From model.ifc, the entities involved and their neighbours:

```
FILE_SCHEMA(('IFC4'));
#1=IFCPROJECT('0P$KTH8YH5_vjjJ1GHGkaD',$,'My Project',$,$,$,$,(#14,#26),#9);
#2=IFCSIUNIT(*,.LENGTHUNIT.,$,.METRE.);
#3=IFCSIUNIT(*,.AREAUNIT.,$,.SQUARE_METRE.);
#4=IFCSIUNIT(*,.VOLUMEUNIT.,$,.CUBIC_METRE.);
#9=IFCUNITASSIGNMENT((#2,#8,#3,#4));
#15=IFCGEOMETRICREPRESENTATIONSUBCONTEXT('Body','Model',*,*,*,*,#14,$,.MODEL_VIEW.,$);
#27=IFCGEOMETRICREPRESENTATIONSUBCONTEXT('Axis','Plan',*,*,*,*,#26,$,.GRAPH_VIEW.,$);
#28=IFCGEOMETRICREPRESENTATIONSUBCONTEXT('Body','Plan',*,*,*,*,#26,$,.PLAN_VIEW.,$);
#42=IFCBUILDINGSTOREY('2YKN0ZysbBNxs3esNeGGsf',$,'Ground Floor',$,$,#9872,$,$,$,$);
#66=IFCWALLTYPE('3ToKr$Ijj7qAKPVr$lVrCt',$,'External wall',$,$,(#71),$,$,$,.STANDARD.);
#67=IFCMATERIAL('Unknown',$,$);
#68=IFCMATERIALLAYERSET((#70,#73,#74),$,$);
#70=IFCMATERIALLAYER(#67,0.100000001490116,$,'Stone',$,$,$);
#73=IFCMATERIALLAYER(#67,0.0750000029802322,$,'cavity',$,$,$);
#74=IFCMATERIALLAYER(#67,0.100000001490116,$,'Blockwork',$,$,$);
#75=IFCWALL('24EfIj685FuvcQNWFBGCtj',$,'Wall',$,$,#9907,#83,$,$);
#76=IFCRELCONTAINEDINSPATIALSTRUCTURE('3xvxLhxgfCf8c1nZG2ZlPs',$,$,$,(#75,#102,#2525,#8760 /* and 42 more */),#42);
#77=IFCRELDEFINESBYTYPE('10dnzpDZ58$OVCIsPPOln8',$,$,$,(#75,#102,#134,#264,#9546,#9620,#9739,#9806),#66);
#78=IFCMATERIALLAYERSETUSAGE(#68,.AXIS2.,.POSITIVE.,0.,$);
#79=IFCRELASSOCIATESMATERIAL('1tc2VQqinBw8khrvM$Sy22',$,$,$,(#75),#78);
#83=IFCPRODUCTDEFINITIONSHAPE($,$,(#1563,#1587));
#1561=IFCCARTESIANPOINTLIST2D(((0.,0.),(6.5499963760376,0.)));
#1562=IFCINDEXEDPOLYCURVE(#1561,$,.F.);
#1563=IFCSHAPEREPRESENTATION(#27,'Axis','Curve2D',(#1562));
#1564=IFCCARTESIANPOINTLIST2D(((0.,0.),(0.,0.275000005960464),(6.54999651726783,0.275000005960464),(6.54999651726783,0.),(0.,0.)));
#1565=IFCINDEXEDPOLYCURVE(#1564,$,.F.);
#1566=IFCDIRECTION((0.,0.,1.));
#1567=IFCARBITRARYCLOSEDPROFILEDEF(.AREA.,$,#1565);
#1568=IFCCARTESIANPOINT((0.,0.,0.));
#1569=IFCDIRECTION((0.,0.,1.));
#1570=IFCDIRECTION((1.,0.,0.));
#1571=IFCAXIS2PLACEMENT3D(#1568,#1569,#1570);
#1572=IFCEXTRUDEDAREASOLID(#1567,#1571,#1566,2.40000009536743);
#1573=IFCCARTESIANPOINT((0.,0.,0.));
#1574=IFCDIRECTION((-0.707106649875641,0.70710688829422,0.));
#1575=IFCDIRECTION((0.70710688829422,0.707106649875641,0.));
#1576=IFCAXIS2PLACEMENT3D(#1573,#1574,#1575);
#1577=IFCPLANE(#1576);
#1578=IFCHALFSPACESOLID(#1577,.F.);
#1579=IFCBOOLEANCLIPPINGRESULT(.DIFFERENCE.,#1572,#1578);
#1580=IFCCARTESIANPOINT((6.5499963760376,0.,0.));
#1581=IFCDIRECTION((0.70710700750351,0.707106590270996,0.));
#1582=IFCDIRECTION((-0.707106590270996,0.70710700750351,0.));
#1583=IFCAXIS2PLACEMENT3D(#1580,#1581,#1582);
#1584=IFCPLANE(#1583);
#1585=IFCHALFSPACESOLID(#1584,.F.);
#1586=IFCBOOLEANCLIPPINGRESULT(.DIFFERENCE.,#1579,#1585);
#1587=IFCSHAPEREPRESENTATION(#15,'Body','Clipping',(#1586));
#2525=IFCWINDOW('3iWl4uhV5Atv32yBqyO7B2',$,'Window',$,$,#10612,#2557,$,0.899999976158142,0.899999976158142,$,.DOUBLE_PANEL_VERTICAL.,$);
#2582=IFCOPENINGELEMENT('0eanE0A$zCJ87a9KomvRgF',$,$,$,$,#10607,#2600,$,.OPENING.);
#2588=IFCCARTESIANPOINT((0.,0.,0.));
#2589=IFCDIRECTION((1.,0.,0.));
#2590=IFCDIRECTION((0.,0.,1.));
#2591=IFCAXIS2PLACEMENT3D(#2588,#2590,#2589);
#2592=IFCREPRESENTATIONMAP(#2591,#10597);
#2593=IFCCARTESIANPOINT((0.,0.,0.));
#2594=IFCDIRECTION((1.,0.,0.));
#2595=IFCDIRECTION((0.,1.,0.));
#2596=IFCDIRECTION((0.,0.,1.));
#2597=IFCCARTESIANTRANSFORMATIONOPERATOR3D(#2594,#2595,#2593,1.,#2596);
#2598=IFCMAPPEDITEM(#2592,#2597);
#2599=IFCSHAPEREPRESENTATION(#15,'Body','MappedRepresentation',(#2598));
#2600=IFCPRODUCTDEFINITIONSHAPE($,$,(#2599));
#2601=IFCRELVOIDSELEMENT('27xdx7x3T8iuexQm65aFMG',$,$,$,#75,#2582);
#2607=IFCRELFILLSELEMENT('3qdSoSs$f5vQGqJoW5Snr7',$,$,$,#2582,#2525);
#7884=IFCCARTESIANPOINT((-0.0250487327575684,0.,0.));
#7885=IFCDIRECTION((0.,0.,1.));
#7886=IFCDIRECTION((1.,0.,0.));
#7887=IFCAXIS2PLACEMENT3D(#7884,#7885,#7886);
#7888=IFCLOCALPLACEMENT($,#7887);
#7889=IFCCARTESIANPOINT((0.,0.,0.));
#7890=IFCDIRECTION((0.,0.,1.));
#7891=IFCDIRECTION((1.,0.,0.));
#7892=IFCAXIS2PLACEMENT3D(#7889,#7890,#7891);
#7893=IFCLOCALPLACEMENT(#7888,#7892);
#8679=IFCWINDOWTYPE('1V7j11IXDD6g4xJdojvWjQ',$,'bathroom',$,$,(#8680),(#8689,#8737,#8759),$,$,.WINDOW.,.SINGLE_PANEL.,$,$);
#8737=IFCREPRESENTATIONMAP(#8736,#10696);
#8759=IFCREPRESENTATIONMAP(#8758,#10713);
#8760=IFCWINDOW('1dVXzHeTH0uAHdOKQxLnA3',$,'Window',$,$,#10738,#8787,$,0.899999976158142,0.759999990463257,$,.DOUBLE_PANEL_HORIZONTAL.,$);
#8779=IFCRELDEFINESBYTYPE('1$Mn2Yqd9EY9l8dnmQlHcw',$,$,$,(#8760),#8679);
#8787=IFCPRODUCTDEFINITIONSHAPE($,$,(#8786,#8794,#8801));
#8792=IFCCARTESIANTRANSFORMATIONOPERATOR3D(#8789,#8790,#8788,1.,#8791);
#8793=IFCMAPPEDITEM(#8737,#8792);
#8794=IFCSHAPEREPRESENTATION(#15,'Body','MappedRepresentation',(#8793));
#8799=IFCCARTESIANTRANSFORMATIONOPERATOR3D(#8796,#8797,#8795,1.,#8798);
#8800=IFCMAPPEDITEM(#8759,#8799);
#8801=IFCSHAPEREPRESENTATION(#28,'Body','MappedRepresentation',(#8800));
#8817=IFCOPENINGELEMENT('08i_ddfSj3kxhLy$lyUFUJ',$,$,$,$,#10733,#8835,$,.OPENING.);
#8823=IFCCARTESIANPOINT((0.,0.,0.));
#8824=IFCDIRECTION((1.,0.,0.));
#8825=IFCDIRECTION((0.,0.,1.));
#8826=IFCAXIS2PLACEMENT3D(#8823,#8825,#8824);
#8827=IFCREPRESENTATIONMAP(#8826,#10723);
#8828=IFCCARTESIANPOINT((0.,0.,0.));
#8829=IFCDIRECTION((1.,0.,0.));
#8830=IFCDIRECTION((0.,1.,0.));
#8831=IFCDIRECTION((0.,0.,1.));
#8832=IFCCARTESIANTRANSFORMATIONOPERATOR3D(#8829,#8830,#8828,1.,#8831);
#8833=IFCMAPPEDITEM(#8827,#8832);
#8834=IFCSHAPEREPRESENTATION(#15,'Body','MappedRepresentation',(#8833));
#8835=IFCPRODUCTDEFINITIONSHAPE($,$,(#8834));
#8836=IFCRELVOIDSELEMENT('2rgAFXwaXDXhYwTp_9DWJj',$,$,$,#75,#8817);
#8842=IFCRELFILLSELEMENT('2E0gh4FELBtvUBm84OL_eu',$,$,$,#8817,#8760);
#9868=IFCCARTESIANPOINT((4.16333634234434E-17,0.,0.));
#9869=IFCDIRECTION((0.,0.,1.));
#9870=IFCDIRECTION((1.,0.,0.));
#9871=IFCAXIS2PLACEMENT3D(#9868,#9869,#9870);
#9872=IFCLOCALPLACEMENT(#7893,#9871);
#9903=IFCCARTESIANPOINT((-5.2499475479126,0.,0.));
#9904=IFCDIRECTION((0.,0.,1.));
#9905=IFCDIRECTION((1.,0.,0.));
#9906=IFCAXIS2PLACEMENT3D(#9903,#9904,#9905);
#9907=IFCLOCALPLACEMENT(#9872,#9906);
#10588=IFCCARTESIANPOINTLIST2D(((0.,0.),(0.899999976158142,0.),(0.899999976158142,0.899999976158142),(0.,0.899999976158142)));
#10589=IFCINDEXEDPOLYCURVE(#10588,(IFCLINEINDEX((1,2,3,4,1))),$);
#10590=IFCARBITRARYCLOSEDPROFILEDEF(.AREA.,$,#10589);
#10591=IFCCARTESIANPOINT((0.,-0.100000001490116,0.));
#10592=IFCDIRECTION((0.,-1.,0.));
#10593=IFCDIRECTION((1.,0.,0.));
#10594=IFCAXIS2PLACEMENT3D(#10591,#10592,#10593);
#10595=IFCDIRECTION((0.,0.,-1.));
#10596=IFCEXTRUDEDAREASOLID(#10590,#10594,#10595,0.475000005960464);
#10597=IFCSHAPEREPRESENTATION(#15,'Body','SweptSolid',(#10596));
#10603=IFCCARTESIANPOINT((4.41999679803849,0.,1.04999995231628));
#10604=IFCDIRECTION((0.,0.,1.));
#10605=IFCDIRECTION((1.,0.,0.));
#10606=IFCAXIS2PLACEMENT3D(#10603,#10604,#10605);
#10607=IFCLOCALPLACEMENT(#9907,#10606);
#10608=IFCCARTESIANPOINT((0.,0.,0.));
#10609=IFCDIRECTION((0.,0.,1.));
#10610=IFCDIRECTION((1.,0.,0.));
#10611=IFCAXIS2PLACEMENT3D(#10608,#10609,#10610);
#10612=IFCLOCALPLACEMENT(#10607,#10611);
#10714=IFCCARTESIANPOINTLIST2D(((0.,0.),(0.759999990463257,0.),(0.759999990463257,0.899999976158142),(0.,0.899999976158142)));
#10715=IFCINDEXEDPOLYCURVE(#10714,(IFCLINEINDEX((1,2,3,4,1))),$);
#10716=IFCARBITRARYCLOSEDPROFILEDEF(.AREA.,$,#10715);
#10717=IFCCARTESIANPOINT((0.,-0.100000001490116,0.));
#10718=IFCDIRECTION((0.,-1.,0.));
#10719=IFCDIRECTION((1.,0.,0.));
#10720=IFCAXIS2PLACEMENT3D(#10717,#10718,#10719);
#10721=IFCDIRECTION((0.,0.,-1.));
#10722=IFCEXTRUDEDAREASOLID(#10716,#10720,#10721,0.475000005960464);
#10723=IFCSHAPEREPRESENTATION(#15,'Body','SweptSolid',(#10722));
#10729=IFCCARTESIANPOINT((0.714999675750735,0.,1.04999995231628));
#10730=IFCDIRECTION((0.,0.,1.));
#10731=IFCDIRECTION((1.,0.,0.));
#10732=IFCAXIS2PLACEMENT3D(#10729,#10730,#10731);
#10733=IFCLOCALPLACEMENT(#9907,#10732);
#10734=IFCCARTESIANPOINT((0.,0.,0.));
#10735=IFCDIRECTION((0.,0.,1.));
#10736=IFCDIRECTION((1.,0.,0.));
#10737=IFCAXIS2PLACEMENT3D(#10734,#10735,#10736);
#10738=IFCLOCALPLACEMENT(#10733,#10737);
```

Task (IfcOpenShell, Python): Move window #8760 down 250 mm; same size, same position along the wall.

```python
import numpy as np
import ifcopenshell
import ifcopenshell.api.geometry
import ifcopenshell.util.placement
import ifcopenshell.util.unit

model = ifcopenshell.open("model.ifc")
unit_scale = ifcopenshell.util.unit.calculate_unit_scale(model)

window = model.by_guid("1dVXzHeTH0uAHdOKQxLnA3")
opening = window.FillsVoids[0].RelatingOpeningElement
dz = -0.25

shift = np.array([0.0, 0.0, dz])
# The window is placed relative to its opening, so it follows when the opening moves.
matrix = ifcopenshell.util.placement.get_local_placement(opening.ObjectPlacement)
matrix[:3, 3] += shift
ifcopenshell.api.geometry.edit_object_placement(
    model, product=opening, matrix=matrix, is_si=False, should_transform_children=True
)

print(f"moved by {dz * unit_scale:+.3f} m")

model.write("model-out.ifc")
```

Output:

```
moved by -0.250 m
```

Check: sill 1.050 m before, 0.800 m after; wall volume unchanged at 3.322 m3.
